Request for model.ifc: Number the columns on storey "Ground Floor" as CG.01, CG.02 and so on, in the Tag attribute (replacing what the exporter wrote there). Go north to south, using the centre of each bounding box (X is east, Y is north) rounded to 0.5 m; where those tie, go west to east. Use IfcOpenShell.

First a look at what the model holds.

```python
import ifcopenshell
import ifcopenshell.util.element
import ifcopenshell.util.placement

model = ifcopenshell.open("model.ifc")
print(model.schema)
storey = next(s for s in model.by_type("IfcBuildingStorey") if s.Name == "Ground Floor")
columns = [e for e in ifcopenshell.util.element.get_decomposition(storey) if e.is_a("IfcColumn")]
for e in sorted(columns, key=lambda e: e.id()):
    origin = ifcopenshell.util.placement.get_local_placement(e.ObjectPlacement)[:3, 3]
    print(e.id(), e.Tag, e.Name, origin.round(2) + 0.0, sep=" | ")
```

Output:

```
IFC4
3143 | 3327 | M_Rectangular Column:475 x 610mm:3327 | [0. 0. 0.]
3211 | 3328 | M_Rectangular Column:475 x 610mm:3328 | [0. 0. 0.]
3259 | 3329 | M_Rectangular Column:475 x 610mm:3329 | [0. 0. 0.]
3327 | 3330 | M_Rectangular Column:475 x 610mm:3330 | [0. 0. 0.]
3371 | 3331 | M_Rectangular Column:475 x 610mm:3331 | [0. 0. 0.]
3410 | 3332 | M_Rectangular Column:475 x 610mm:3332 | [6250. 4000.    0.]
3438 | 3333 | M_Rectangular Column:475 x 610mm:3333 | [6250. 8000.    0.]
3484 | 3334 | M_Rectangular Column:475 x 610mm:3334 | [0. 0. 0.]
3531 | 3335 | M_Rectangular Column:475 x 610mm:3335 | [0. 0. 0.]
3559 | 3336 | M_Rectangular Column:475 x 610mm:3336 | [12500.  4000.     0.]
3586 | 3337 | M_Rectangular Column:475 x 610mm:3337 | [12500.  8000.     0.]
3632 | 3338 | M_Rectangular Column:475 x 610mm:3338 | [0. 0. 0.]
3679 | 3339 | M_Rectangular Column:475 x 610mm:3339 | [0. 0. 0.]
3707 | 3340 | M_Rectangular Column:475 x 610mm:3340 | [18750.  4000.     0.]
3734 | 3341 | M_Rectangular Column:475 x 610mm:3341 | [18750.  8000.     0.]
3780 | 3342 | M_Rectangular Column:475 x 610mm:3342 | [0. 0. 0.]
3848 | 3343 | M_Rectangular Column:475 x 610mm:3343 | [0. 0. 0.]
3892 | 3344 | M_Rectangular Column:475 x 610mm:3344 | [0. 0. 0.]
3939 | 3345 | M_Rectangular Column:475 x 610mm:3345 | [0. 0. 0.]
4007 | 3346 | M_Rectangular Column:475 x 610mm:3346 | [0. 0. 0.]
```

```python
import ifcopenshell
import ifcopenshell.geom
import ifcopenshell.util.element
import ifcopenshell.util.shape

model = ifcopenshell.open("model.ifc")
settings = ifcopenshell.geom.settings()
settings.set("use-world-coords", True)


def centre(element):
    shape = ifcopenshell.geom.create_shape(settings, element)
    return ifcopenshell.util.shape.get_bbox_centroid(shape.geometry)


storey = next(s for s in model.by_type("IfcBuildingStorey") if s.Name == "Ground Floor")
columns = [e for e in ifcopenshell.util.element.get_decomposition(storey) if e.is_a("IfcColumn")]

# Insertion points can sit at a corner or the storey origin, so sort by the geometry (in metres).
centres = {e: centre(e) for e in columns}
columns.sort(key=lambda e: (-round(centres[e][1] / 0.5), centres[e][0]))

for i, e in enumerate(columns, start=1):
    number = f"CG.{i:02d}"
    e.Tag = number
    print(e.id(), number)

model.write("model_updated.ifc")
```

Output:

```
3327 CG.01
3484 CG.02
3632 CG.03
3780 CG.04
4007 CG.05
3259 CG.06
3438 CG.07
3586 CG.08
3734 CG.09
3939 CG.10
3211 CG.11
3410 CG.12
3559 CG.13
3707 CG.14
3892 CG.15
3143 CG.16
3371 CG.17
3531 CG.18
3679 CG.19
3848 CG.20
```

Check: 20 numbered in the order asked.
